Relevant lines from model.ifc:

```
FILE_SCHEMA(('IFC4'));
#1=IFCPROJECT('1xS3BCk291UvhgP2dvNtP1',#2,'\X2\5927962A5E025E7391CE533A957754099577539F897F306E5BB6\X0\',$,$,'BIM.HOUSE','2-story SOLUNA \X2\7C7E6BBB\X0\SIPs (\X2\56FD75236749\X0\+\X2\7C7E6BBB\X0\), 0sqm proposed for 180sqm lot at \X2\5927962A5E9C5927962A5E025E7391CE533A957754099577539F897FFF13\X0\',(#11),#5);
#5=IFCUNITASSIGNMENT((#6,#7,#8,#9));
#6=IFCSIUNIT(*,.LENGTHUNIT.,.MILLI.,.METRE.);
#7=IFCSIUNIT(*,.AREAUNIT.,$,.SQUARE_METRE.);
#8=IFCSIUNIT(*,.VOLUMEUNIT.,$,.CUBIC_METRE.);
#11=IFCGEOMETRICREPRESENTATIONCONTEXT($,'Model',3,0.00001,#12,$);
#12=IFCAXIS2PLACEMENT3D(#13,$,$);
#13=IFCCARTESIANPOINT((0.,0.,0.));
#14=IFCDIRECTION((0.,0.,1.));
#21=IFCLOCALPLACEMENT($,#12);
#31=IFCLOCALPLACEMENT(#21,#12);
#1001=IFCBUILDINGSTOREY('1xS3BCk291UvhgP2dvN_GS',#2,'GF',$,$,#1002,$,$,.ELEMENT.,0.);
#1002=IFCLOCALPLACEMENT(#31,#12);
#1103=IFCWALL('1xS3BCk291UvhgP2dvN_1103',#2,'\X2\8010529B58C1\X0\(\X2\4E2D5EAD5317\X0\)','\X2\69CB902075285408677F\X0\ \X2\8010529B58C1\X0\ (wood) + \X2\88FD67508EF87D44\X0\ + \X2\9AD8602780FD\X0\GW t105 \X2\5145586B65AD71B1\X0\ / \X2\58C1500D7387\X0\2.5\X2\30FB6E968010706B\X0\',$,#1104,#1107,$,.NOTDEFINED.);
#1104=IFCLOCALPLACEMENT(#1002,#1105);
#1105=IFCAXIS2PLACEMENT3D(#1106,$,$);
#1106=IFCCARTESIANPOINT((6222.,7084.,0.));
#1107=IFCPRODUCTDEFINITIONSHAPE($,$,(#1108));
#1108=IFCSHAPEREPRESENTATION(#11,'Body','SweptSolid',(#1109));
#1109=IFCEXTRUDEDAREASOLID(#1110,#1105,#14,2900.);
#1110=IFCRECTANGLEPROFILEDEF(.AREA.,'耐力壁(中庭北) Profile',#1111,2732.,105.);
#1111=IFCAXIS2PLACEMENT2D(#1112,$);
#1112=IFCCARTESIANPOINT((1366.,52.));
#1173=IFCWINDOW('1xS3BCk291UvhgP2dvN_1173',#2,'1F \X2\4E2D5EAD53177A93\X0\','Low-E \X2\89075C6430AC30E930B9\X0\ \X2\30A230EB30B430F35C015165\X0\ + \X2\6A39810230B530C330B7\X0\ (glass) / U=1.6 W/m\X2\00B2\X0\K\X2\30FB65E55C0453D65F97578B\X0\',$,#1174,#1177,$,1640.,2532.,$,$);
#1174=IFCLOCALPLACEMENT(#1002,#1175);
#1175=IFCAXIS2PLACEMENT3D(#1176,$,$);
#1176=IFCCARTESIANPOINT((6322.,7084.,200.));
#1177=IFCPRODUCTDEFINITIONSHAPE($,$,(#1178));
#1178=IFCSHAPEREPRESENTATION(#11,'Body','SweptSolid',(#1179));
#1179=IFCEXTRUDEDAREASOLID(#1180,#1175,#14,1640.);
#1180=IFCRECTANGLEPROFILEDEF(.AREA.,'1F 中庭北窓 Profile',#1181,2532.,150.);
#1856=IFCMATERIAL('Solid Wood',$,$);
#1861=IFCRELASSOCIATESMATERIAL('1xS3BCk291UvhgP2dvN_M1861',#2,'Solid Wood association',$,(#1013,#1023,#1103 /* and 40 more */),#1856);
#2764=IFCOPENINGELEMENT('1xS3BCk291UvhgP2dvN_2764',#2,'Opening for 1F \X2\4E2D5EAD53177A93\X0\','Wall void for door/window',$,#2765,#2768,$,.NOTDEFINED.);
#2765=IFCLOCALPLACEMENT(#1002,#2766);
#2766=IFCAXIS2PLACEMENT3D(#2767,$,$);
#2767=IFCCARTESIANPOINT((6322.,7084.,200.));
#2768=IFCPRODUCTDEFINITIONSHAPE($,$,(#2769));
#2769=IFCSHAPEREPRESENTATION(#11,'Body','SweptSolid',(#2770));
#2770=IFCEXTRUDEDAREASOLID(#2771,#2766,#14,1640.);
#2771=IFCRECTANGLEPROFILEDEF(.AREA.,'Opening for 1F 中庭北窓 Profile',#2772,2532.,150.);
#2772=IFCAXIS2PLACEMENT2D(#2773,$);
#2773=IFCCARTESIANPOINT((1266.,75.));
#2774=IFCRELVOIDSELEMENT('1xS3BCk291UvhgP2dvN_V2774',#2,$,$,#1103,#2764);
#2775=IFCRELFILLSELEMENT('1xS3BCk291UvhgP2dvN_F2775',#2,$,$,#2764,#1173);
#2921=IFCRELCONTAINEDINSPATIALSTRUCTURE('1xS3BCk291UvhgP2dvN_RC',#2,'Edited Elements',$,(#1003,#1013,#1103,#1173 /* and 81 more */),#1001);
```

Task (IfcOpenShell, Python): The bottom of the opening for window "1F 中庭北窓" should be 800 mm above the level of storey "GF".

```python
import numpy as np
import ifcopenshell
import ifcopenshell.api.geometry
import ifcopenshell.geom
import ifcopenshell.util.element
import ifcopenshell.util.placement
import ifcopenshell.util.shape
import ifcopenshell.util.unit

model = ifcopenshell.open("model.ifc")
unit_scale = ifcopenshell.util.unit.calculate_unit_scale(model)

window = model.by_guid("1xS3BCk291UvhgP2dvN_1173")
opening = window.FillsVoids[0].RelatingOpeningElement
storey = ifcopenshell.util.element.get_container(window, ifc_class="IfcBuildingStorey")
level = ifcopenshell.util.placement.get_local_placement(storey.ObjectPlacement)[2, 3]

# The opening's origin need not be at the sill, so measure its lowest point.
shape = ifcopenshell.geom.create_shape(ifcopenshell.geom.settings(), opening)
bottom = ifcopenshell.util.shape.get_shape_bottom_elevation(shape, shape.geometry) / unit_scale
dz = level + 0.8 / unit_scale - bottom

shift = np.array([0.0, 0.0, dz])
# The window is not placed relative to its opening, so move both.
for product in (opening, window):
    matrix = ifcopenshell.util.placement.get_local_placement(product.ObjectPlacement)
    matrix[:3, 3] += shift
    ifcopenshell.api.geometry.edit_object_placement(model, product=product, matrix=matrix, is_si=False)

print(f"moved by {dz * unit_scale:+.3f} m")

model.write("model-out.ifc")
```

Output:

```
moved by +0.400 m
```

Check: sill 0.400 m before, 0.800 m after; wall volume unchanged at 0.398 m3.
